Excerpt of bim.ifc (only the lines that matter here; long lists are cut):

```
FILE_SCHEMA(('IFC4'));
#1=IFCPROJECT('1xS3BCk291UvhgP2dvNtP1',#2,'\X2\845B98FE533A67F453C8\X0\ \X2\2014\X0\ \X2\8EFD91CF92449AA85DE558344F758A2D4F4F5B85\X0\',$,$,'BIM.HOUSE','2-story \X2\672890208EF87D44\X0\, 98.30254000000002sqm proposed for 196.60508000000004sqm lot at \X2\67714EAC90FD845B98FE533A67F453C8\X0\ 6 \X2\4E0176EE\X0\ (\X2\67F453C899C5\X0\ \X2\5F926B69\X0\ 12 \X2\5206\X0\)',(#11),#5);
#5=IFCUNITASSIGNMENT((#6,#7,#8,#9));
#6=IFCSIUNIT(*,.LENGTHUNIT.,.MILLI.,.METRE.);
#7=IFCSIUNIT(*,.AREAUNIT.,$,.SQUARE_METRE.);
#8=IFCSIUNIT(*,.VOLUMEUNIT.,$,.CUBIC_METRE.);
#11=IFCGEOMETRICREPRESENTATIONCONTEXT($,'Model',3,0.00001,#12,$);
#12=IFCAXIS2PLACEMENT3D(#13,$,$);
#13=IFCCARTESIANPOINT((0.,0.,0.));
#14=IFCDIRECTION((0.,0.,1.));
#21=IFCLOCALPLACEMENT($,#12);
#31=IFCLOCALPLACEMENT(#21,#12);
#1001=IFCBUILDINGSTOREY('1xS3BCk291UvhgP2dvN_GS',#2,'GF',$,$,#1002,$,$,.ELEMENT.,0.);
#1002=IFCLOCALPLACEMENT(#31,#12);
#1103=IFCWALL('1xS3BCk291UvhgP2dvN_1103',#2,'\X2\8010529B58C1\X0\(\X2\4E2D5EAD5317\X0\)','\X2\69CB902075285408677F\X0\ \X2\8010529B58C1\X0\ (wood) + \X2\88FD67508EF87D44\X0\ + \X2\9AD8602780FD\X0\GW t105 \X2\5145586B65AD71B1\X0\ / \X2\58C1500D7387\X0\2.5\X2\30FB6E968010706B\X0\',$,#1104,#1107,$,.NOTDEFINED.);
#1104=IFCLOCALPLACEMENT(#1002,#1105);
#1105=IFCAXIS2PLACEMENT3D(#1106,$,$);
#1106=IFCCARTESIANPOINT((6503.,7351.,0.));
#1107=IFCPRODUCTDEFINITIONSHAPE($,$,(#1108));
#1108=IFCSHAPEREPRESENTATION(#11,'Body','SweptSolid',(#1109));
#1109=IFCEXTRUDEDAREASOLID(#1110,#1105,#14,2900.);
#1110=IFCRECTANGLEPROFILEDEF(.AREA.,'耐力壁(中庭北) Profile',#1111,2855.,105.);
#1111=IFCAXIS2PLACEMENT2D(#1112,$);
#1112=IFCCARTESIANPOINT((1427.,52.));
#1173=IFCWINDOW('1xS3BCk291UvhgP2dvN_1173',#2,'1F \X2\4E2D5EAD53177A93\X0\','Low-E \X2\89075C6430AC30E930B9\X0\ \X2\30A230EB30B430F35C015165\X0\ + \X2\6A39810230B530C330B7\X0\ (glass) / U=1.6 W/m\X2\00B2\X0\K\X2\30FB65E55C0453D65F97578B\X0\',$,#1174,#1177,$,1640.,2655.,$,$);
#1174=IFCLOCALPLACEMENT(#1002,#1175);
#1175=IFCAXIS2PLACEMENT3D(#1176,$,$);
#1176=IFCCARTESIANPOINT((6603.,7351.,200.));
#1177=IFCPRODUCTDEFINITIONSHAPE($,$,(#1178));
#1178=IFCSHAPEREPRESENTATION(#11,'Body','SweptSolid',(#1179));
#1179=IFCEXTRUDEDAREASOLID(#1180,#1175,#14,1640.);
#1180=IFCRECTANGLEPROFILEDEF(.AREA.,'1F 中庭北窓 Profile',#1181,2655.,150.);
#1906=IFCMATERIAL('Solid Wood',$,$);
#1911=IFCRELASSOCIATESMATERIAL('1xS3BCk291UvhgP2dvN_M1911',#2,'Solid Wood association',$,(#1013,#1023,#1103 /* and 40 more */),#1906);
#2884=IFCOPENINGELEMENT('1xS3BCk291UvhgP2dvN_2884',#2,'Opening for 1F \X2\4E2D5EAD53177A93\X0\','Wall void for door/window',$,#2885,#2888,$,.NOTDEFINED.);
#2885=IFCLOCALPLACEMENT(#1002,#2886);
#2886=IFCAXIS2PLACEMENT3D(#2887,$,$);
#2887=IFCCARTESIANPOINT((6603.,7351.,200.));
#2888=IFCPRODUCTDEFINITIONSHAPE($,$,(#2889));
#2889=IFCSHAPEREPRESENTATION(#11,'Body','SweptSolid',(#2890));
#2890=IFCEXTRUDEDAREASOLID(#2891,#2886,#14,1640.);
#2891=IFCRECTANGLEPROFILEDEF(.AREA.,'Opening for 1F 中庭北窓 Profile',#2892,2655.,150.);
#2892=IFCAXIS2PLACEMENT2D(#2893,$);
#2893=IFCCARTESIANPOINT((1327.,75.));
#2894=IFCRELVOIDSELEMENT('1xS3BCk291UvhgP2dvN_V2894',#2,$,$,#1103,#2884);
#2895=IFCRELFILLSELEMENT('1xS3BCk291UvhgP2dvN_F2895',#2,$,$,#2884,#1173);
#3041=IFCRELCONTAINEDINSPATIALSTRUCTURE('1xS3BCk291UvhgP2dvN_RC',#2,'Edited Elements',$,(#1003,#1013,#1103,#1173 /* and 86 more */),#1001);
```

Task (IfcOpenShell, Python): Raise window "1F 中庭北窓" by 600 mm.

```python
import numpy as np
import ifcopenshell
import ifcopenshell.api.geometry
import ifcopenshell.util.placement
import ifcopenshell.util.unit

model = ifcopenshell.open("bim.ifc")
unit_scale = ifcopenshell.util.unit.calculate_unit_scale(model)

window = model.by_guid("1xS3BCk291UvhgP2dvN_1173")
opening = window.FillsVoids[0].RelatingOpeningElement
dz = 0.6 / unit_scale

shift = np.array([0.0, 0.0, dz])
# The window is not placed relative to its opening, so move both.
for product in (opening, window):
    matrix = ifcopenshell.util.placement.get_local_placement(product.ObjectPlacement)
    matrix[:3, 3] += shift
    ifcopenshell.api.geometry.edit_object_placement(model, product=product, matrix=matrix, is_si=False)

print(f"moved by {dz * unit_scale:+.3f} m")

model.write("bim_v2.ifc")
```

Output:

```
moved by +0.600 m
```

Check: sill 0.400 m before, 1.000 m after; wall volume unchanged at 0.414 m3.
